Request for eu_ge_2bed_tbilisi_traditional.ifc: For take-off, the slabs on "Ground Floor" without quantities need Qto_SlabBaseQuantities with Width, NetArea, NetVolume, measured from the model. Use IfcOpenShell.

First a look at what the model holds.

```python
import ifcopenshell
import ifcopenshell.util.element
import ifcopenshell.util.unit

model = ifcopenshell.open("eu_ge_2bed_tbilisi_traditional.ifc")
print(model.schema)
for unit_type in ("LENGTHUNIT", "AREAUNIT", "VOLUMEUNIT"):
    print(unit_type, ifcopenshell.util.unit.calculate_unit_scale(model, unit_type))
storey = next(s for s in model.by_type("IfcBuildingStorey") if s.Name == "Ground Floor")
slabs = [e for e in ifcopenshell.util.element.get_decomposition(storey) if e.is_a("IfcSlab")]
for e in sorted(slabs, key=lambda e: e.id()):
    print(e.id(), e.is_a(), e.Name, list(ifcopenshell.util.element.get_psets(e, qtos_only=True)), sep=" | ")
```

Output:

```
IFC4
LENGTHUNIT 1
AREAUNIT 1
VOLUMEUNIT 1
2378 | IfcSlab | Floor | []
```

```python
import ifcopenshell
import ifcopenshell.api.pset
import ifcopenshell.geom
import ifcopenshell.util.element
import ifcopenshell.util.shape
import ifcopenshell.util.unit

model = ifcopenshell.open("eu_ge_2bed_tbilisi_traditional.ifc")
unit_scale = ifcopenshell.util.unit.calculate_unit_scale(model)
area_scale = ifcopenshell.util.unit.calculate_unit_scale(model, "AREAUNIT")
volume_scale = ifcopenshell.util.unit.calculate_unit_scale(model, "VOLUMEUNIT")
settings = ifcopenshell.geom.settings()

storey = next(s for s in model.by_type("IfcBuildingStorey") if s.Name == "Ground Floor")
slabs = [e for e in ifcopenshell.util.element.get_decomposition(storey) if e.is_a("IfcSlab")]

for e in sorted(slabs, key=lambda e: e.id()):
    if ifcopenshell.util.element.get_psets(e, qtos_only=True, should_inherit=False):
        continue
    # Geometry comes back in metres, in the element's own axes.
    shape = ifcopenshell.geom.create_shape(settings, e)
    values = {
        "Width": ifcopenshell.util.shape.get_z(shape.geometry) / unit_scale,
        "NetArea": ifcopenshell.util.shape.get_footprint_area(shape.geometry) / area_scale,
        "NetVolume": ifcopenshell.util.shape.get_volume(shape.geometry) / volume_scale,
    }
    qto = ifcopenshell.api.pset.add_qto(model, product=e, name="Qto_SlabBaseQuantities")
    ifcopenshell.api.pset.edit_qto(model, qto=qto, properties=values)
    print(e.id(), {k: round(v, 3) for k, v in values.items()})

model.write("eu_ge_2bed_tbilisi_traditional_edited.ifc")
```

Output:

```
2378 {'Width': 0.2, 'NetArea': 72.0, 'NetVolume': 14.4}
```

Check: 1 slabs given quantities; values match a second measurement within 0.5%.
